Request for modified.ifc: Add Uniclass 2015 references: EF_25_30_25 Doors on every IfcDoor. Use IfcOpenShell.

First a look at what the model holds.

```python
import ifcopenshell

model = ifcopenshell.open("modified.ifc")
print(model.schema)
print("classifications:", [c.Name for c in model.by_type("IfcClassification")])
for ifc_class in ("IfcDoor", "IfcRoof", "IfcStair", "IfcWall", "IfcWindow"):
    print(ifc_class, len(model.by_type(ifc_class)))
```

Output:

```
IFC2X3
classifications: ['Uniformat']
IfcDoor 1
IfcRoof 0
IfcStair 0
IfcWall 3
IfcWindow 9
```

```python
import ifcopenshell
import ifcopenshell.api.classification

model = ifcopenshell.open("modified.ifc")

# IFC2X3 requires Source and Edition and has no link from the project to the system.
system = model.create_entity("IfcClassification", Source="NBS", Edition="2015", Name="Uniclass 2015")

codes = {
    "IfcDoor": ("EF_25_30_25", "Doors"),
}
for ifc_class, (code, name) in codes.items():
    products = model.by_type(ifc_class)
    ifcopenshell.api.classification.add_reference(
        model, products=products, classification=system, identification=code, name=name
    )
    print(code, len(products))

model.write("modified_updated.ifc")
```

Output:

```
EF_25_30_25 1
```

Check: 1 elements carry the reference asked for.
